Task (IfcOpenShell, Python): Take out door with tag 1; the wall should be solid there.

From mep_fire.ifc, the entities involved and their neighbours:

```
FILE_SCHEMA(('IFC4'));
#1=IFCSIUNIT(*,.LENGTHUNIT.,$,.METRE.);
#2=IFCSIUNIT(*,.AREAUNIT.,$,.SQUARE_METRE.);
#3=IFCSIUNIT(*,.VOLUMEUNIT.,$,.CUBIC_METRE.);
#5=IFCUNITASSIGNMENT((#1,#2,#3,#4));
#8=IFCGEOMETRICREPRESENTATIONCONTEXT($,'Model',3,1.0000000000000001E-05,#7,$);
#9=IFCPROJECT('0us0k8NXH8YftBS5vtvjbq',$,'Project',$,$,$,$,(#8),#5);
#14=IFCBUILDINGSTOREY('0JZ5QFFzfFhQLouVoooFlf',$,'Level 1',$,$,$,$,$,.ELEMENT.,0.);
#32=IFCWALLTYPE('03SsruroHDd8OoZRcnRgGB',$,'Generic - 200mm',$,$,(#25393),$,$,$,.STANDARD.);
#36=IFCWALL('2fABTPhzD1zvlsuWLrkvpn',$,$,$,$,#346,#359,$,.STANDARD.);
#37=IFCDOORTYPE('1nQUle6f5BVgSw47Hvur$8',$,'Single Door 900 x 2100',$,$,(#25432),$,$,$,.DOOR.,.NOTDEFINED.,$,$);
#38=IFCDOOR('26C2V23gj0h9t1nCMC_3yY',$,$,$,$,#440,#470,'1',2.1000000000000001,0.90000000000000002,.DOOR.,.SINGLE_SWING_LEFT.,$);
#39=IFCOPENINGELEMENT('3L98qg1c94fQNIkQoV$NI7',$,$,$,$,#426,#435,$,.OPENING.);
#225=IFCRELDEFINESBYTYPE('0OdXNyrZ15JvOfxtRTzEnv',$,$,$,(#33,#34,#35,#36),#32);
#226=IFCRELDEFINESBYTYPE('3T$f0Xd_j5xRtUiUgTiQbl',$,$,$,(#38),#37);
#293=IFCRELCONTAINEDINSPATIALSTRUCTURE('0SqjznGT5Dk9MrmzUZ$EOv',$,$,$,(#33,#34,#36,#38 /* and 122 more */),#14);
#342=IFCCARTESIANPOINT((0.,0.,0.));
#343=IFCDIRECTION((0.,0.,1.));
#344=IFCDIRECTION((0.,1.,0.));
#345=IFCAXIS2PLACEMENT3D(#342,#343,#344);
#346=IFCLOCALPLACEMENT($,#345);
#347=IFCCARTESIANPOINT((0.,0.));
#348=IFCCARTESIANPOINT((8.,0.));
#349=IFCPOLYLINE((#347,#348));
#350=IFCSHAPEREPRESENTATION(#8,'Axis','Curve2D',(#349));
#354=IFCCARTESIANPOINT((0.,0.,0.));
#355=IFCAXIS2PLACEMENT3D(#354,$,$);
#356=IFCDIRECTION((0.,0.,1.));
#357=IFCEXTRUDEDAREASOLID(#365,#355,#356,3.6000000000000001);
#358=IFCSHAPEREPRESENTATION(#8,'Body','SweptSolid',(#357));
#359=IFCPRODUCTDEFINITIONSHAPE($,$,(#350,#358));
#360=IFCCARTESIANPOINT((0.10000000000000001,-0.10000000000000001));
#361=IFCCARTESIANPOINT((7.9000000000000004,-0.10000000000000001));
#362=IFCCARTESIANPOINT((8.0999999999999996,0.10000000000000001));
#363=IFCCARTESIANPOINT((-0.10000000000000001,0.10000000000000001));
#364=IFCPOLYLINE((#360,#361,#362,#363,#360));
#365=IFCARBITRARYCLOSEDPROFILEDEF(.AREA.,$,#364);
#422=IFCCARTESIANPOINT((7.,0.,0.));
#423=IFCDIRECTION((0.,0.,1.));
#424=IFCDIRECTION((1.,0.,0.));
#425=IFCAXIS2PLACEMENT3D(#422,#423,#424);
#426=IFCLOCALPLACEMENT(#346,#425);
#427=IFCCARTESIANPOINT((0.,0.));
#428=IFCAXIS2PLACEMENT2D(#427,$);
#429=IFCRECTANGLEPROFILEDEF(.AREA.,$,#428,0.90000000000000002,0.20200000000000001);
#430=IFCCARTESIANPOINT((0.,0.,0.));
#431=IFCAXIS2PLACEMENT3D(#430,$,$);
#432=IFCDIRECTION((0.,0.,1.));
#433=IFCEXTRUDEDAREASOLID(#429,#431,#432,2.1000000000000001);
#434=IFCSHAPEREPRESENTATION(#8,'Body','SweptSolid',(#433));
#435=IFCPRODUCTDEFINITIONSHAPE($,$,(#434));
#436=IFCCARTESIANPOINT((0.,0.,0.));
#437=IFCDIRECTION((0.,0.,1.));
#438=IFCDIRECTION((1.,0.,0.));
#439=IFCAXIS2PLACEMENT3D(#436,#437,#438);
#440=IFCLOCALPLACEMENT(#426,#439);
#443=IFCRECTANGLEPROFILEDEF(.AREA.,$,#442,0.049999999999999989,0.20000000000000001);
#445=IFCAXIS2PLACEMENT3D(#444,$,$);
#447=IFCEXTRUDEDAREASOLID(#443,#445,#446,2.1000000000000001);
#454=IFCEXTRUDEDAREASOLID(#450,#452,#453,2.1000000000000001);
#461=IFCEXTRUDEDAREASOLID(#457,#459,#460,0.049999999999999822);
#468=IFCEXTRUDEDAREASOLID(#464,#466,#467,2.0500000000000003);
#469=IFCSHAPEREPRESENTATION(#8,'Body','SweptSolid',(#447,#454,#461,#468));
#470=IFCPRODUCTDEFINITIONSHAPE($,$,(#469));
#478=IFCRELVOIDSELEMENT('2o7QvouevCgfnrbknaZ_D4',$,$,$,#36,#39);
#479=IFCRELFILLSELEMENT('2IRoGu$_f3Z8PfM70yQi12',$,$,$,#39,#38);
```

```python
import ifcopenshell
import ifcopenshell.api.feature
import ifcopenshell.api.root
import ifcopenshell.geom
import ifcopenshell.util.shape

model = ifcopenshell.open("mep_fire.ifc")
settings = ifcopenshell.geom.settings()


def volume(element):
    """Net volume in cubic metres, openings subtracted."""
    shape = ifcopenshell.geom.create_shape(settings, element)
    return ifcopenshell.util.shape.get_volume(shape.geometry)


door = model.by_id(38)
opening = door.FillsVoids[0].RelatingOpeningElement
wall = opening.VoidsElements[0].RelatingBuildingElement
before = volume(wall)

ifcopenshell.api.root.remove_product(model, product=door)
ifcopenshell.api.feature.remove_feature(model, feature=opening)

after = volume(wall)

print(f"wall volume {before:.3f} -> {after:.3f} m3")

model.write("mep_fire_updated.ifc")
```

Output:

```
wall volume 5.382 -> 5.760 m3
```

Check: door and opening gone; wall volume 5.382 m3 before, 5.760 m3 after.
